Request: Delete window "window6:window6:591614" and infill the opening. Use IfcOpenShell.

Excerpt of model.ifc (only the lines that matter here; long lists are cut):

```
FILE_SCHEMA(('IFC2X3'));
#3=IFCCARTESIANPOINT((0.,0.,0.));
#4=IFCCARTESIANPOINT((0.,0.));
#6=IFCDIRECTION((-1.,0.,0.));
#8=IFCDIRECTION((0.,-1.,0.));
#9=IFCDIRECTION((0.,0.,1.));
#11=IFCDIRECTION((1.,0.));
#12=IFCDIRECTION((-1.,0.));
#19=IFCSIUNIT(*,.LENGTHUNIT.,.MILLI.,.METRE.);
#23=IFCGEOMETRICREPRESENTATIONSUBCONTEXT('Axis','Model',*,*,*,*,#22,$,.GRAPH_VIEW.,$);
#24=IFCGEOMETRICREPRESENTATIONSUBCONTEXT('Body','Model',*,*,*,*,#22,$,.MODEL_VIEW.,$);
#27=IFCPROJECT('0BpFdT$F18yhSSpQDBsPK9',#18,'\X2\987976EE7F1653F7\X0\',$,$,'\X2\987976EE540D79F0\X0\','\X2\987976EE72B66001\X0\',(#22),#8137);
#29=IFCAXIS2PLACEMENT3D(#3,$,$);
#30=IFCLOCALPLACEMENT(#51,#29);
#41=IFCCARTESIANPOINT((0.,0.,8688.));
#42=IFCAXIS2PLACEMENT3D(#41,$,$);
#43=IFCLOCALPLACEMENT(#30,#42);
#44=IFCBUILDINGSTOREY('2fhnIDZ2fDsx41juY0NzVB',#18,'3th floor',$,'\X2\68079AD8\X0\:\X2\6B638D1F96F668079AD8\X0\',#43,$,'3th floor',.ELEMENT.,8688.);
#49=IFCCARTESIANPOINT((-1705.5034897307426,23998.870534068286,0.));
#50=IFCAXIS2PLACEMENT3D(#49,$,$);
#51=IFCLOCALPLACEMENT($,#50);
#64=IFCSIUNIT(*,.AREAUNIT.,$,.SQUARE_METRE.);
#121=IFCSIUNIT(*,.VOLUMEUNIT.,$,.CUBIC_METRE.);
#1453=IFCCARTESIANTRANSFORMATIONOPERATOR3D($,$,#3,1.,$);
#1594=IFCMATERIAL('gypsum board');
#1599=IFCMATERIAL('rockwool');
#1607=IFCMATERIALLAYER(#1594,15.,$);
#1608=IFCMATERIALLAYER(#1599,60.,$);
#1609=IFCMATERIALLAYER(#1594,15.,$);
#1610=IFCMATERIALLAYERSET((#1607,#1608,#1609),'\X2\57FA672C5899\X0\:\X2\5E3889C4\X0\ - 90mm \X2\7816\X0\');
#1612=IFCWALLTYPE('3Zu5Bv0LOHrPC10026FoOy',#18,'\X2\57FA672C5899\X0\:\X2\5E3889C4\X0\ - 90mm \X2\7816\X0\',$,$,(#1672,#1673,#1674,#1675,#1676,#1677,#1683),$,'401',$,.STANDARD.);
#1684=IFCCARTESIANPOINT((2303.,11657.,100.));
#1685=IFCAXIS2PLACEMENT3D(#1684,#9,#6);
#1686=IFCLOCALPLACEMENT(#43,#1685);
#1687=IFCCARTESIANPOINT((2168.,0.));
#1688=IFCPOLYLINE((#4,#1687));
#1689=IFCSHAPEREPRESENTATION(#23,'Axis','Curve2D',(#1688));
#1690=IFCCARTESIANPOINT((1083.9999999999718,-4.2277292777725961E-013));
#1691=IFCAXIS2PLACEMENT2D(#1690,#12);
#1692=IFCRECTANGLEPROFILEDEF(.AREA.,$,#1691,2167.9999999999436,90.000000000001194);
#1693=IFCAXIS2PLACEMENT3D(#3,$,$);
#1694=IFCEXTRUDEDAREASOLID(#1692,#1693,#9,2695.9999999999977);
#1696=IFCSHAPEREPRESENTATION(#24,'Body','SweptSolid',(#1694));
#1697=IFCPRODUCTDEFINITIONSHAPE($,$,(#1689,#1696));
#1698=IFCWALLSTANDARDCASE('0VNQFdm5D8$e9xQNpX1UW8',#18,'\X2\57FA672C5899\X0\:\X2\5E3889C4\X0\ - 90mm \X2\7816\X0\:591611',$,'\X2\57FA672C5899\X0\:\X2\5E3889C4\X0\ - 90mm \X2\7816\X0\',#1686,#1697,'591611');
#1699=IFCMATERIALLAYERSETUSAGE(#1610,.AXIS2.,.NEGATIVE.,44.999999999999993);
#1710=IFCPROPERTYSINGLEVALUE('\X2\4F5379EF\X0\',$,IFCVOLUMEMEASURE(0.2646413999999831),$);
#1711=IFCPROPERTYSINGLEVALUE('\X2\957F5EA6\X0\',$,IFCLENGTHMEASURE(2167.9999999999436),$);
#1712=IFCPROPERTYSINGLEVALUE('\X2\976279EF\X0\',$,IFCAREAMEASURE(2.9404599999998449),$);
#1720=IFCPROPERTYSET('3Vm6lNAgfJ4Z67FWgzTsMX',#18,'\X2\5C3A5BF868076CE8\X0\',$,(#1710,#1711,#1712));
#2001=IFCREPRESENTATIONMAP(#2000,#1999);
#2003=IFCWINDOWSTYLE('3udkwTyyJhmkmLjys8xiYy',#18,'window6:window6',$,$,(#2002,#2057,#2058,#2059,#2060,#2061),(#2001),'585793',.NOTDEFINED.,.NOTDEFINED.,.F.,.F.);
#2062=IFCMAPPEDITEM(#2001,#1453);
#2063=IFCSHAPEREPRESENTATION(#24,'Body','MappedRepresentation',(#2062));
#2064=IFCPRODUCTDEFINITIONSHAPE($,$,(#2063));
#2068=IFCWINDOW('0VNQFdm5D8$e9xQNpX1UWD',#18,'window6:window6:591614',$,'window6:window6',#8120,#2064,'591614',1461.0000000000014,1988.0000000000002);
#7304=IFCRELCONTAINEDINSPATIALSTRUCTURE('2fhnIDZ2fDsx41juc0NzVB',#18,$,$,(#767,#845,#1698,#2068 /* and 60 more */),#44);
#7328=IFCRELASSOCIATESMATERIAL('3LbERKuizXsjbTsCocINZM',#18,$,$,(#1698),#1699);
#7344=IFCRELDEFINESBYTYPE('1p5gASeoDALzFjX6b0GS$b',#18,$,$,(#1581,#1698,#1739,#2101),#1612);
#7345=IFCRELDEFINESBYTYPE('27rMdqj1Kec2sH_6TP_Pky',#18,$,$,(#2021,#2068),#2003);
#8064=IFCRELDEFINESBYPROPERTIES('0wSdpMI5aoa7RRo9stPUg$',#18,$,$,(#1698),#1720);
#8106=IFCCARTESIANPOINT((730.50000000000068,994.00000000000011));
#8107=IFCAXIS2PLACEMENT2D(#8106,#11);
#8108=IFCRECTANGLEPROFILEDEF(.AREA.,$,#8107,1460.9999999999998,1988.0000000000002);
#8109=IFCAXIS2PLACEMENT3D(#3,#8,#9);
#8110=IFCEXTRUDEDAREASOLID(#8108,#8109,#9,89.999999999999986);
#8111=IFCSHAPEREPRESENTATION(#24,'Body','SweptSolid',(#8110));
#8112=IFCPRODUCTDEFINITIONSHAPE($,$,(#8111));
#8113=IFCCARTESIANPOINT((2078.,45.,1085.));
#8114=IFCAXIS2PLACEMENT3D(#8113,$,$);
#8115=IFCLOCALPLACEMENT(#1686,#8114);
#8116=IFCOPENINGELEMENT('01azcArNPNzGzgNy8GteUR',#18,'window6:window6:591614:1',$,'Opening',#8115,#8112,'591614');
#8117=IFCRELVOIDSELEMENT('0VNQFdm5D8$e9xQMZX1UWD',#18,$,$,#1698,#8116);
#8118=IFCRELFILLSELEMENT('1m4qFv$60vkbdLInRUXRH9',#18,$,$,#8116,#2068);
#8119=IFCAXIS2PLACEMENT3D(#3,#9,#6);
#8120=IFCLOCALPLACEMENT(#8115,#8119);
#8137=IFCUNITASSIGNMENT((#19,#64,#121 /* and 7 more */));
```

```python
import ifcopenshell
import ifcopenshell.api.feature
import ifcopenshell.api.pset
import ifcopenshell.api.root
import ifcopenshell.geom
import ifcopenshell.util.element
import ifcopenshell.util.shape
import ifcopenshell.util.unit

model = ifcopenshell.open("model.ifc")
area_scale = ifcopenshell.util.unit.calculate_unit_scale(model, "AREAUNIT")
volume_scale = ifcopenshell.util.unit.calculate_unit_scale(model, "VOLUMEUNIT")
settings = ifcopenshell.geom.settings()


def volume(element):
    """Net volume in cubic metres, openings subtracted."""
    shape = ifcopenshell.geom.create_shape(settings, element)
    return ifcopenshell.util.shape.get_volume(shape.geometry)


window = model.by_guid("0VNQFdm5D8$e9xQNpX1UWD")
opening = window.FillsVoids[0].RelatingOpeningElement
wall = opening.VoidsElements[0].RelatingBuildingElement
before = volume(wall)

ifcopenshell.api.root.remove_product(model, product=window)
ifcopenshell.api.feature.remove_feature(model, feature=opening)

after = volume(wall)
thickness = 0.09  # wall thickness in metres

# Update the wall's stored quantities.
pset = model.by_id(ifcopenshell.util.element.get_pset(wall, "尺寸标注", should_inherit=False)["id"])
ifcopenshell.api.pset.edit_pset(model, pset=pset, properties={
    "体积": model.create_entity("IfcVolumeMeasure", after / volume_scale),
    "面积": model.create_entity("IfcAreaMeasure", after / thickness / area_scale),
})

print(f"wall volume {before:.3f} -> {after:.3f} m3")

model.write("model_updated.ifc")
```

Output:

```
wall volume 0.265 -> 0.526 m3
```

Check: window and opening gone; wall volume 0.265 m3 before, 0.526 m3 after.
